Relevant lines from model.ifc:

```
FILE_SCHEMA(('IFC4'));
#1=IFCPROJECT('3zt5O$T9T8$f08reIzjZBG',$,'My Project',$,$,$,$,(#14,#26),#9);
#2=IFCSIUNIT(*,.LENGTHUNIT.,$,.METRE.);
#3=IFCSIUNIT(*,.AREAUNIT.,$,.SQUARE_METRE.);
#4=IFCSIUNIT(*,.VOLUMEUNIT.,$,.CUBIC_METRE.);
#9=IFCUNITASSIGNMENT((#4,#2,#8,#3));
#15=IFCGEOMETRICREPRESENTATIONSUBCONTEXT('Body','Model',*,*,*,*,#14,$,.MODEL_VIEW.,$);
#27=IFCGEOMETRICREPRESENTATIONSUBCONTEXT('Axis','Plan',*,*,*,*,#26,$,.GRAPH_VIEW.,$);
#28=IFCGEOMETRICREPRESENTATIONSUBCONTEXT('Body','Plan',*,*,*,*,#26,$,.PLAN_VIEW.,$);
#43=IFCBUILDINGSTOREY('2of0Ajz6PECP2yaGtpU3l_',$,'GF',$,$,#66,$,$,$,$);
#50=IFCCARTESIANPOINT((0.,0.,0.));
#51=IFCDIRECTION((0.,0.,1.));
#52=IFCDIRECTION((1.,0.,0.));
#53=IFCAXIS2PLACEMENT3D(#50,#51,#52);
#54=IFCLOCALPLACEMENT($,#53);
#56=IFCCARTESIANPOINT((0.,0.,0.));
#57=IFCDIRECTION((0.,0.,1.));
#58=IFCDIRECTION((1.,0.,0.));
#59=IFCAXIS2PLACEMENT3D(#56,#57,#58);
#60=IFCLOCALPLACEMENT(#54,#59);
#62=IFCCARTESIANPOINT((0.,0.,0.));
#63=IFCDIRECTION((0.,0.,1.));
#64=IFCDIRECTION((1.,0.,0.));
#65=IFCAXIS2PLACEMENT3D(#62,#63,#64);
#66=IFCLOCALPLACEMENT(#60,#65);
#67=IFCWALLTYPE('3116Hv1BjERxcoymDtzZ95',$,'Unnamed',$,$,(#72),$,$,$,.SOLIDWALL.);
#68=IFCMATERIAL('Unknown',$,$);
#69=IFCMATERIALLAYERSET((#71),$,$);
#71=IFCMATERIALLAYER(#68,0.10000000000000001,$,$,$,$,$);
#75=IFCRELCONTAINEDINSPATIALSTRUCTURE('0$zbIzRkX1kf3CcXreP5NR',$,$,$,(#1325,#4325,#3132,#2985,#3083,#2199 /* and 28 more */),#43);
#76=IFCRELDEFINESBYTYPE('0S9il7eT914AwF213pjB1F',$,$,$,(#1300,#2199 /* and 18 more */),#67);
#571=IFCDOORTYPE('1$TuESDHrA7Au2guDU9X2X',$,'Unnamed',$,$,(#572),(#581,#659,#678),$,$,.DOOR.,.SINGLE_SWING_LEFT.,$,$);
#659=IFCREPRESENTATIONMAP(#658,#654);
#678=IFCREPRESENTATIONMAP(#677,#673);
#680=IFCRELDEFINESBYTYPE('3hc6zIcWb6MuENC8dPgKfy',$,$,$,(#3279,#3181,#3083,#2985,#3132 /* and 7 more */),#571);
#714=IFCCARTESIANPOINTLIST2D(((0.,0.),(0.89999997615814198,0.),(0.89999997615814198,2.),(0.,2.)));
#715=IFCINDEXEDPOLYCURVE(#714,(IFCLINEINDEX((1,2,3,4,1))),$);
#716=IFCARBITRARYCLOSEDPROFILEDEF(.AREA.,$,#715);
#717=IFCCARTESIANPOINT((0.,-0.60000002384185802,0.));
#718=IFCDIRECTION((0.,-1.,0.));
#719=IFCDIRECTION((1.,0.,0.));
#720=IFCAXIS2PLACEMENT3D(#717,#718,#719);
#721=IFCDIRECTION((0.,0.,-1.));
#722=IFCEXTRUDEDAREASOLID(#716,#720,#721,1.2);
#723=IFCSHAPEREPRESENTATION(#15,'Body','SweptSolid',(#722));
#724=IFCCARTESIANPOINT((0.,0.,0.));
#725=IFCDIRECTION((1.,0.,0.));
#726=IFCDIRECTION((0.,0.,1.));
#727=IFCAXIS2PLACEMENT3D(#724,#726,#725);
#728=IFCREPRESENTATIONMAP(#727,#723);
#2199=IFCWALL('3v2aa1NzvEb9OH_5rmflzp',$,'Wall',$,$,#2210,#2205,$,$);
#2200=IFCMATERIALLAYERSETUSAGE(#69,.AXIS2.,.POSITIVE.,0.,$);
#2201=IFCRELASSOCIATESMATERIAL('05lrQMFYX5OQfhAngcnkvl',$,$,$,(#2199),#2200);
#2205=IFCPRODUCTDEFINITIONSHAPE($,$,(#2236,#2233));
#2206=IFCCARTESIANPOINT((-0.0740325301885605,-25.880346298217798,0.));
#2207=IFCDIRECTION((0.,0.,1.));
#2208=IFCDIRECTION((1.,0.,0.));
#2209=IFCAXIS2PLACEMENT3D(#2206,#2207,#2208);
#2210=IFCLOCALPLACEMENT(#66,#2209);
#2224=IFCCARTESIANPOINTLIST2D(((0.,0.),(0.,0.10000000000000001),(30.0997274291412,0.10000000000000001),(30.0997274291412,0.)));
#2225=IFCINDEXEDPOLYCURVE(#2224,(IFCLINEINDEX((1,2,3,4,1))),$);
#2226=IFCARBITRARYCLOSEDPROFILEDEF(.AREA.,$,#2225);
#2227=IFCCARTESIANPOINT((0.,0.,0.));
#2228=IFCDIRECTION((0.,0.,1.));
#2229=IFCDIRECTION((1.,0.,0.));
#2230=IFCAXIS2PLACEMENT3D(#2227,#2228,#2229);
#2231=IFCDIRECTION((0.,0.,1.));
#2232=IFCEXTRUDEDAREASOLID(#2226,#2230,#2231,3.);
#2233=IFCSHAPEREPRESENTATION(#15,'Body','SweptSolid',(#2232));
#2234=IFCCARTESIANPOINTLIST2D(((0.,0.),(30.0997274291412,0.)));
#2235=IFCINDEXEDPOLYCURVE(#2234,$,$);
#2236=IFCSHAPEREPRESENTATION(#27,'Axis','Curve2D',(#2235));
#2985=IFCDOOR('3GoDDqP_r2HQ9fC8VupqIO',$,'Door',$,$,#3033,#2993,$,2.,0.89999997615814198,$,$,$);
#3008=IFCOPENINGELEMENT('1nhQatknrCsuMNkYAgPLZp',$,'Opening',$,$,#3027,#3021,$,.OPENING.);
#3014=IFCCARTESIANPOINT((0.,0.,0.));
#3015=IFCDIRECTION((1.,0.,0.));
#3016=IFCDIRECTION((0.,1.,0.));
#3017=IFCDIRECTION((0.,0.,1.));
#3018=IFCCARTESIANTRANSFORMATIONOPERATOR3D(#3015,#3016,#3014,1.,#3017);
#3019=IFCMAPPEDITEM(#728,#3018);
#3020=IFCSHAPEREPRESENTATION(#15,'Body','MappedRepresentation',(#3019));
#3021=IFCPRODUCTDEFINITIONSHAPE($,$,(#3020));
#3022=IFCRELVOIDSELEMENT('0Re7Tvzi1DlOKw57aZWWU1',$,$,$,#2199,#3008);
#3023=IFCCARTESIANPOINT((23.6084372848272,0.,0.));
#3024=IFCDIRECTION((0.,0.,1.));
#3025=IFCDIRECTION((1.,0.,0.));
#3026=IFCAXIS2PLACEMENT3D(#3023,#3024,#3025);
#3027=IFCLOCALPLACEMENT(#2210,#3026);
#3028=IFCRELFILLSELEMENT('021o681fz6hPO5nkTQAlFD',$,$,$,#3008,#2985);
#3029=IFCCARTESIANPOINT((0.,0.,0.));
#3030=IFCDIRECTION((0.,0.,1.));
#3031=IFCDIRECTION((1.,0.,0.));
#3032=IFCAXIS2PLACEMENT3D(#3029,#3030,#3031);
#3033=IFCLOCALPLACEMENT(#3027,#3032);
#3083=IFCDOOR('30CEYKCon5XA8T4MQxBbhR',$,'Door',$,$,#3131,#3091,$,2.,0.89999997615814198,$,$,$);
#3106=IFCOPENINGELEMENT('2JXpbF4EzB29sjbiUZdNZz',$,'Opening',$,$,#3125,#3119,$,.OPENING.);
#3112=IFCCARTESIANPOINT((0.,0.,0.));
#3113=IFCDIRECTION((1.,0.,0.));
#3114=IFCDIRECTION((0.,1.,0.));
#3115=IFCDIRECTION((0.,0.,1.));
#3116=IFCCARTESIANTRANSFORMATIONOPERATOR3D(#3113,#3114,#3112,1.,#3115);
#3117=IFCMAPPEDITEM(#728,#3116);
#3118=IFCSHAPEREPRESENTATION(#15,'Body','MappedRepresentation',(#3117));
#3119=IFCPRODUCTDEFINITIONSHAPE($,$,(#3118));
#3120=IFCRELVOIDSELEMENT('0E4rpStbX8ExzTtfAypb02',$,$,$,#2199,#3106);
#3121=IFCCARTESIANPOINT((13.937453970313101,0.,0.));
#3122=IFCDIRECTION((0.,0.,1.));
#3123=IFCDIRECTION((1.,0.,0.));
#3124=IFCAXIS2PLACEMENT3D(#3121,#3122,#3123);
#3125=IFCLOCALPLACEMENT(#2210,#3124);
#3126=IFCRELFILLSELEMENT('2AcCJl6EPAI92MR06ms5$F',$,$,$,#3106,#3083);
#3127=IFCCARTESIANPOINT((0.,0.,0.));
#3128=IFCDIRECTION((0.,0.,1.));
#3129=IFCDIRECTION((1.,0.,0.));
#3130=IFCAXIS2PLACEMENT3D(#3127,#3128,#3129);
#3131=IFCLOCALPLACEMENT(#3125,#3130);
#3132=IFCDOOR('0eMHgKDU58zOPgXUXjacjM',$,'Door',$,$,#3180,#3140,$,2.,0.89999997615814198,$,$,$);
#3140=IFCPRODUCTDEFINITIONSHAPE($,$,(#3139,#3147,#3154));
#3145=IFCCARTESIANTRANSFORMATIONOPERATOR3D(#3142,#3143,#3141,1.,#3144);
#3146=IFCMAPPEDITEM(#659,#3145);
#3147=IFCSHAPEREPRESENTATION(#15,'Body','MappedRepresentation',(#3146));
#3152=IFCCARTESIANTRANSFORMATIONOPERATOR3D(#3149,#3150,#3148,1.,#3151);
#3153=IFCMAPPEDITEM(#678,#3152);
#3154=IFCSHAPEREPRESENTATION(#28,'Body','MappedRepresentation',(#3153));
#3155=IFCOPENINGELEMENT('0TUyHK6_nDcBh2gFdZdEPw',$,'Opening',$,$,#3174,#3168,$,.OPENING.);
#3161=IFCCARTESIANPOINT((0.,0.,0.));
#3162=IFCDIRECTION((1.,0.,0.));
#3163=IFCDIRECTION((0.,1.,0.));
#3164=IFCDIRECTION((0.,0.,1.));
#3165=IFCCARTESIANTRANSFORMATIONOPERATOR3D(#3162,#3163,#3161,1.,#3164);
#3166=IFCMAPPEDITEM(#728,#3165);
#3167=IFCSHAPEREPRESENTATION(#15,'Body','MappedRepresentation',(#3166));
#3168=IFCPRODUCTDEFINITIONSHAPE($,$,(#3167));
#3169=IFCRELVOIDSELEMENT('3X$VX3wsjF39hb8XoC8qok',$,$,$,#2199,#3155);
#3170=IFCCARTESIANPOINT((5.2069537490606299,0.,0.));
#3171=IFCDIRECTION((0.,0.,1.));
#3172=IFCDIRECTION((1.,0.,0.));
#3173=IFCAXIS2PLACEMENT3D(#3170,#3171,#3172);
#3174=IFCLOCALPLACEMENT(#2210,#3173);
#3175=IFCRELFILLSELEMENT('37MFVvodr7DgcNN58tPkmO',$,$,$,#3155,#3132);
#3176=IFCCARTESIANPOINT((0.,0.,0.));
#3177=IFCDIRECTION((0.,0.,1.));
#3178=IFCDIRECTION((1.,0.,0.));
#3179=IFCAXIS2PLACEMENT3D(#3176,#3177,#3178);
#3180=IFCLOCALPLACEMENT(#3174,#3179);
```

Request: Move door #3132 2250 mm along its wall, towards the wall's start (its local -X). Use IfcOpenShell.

```python
import ifcopenshell
import ifcopenshell.api.geometry
import ifcopenshell.util.placement

model = ifcopenshell.open("model.ifc")

door = model.by_guid("0eMHgKDU58zOPgXUXjacjM")
opening = door.FillsVoids[0].RelatingOpeningElement
wall = opening.VoidsElements[0].RelatingBuildingElement

wall_matrix = ifcopenshell.util.placement.get_local_placement(wall.ObjectPlacement)
shift = wall_matrix[:3, 0] * -2.25
before = ifcopenshell.util.placement.get_local_placement(door.ObjectPlacement)[:3, 3].copy()

# The door is placed relative to its opening, so it follows when the opening moves.
matrix = ifcopenshell.util.placement.get_local_placement(opening.ObjectPlacement)
matrix[:3, 3] += shift
ifcopenshell.api.geometry.edit_object_placement(
    model, product=opening, matrix=matrix, is_si=False, should_transform_children=True
)

after = ifcopenshell.util.placement.get_local_placement(door.ObjectPlacement)[:3, 3]
print("door moved by", (after - before).round(3) + 0.0)

model.write("model_updated.ifc")
```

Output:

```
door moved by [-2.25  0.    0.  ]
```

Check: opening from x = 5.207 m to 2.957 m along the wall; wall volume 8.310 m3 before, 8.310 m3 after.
